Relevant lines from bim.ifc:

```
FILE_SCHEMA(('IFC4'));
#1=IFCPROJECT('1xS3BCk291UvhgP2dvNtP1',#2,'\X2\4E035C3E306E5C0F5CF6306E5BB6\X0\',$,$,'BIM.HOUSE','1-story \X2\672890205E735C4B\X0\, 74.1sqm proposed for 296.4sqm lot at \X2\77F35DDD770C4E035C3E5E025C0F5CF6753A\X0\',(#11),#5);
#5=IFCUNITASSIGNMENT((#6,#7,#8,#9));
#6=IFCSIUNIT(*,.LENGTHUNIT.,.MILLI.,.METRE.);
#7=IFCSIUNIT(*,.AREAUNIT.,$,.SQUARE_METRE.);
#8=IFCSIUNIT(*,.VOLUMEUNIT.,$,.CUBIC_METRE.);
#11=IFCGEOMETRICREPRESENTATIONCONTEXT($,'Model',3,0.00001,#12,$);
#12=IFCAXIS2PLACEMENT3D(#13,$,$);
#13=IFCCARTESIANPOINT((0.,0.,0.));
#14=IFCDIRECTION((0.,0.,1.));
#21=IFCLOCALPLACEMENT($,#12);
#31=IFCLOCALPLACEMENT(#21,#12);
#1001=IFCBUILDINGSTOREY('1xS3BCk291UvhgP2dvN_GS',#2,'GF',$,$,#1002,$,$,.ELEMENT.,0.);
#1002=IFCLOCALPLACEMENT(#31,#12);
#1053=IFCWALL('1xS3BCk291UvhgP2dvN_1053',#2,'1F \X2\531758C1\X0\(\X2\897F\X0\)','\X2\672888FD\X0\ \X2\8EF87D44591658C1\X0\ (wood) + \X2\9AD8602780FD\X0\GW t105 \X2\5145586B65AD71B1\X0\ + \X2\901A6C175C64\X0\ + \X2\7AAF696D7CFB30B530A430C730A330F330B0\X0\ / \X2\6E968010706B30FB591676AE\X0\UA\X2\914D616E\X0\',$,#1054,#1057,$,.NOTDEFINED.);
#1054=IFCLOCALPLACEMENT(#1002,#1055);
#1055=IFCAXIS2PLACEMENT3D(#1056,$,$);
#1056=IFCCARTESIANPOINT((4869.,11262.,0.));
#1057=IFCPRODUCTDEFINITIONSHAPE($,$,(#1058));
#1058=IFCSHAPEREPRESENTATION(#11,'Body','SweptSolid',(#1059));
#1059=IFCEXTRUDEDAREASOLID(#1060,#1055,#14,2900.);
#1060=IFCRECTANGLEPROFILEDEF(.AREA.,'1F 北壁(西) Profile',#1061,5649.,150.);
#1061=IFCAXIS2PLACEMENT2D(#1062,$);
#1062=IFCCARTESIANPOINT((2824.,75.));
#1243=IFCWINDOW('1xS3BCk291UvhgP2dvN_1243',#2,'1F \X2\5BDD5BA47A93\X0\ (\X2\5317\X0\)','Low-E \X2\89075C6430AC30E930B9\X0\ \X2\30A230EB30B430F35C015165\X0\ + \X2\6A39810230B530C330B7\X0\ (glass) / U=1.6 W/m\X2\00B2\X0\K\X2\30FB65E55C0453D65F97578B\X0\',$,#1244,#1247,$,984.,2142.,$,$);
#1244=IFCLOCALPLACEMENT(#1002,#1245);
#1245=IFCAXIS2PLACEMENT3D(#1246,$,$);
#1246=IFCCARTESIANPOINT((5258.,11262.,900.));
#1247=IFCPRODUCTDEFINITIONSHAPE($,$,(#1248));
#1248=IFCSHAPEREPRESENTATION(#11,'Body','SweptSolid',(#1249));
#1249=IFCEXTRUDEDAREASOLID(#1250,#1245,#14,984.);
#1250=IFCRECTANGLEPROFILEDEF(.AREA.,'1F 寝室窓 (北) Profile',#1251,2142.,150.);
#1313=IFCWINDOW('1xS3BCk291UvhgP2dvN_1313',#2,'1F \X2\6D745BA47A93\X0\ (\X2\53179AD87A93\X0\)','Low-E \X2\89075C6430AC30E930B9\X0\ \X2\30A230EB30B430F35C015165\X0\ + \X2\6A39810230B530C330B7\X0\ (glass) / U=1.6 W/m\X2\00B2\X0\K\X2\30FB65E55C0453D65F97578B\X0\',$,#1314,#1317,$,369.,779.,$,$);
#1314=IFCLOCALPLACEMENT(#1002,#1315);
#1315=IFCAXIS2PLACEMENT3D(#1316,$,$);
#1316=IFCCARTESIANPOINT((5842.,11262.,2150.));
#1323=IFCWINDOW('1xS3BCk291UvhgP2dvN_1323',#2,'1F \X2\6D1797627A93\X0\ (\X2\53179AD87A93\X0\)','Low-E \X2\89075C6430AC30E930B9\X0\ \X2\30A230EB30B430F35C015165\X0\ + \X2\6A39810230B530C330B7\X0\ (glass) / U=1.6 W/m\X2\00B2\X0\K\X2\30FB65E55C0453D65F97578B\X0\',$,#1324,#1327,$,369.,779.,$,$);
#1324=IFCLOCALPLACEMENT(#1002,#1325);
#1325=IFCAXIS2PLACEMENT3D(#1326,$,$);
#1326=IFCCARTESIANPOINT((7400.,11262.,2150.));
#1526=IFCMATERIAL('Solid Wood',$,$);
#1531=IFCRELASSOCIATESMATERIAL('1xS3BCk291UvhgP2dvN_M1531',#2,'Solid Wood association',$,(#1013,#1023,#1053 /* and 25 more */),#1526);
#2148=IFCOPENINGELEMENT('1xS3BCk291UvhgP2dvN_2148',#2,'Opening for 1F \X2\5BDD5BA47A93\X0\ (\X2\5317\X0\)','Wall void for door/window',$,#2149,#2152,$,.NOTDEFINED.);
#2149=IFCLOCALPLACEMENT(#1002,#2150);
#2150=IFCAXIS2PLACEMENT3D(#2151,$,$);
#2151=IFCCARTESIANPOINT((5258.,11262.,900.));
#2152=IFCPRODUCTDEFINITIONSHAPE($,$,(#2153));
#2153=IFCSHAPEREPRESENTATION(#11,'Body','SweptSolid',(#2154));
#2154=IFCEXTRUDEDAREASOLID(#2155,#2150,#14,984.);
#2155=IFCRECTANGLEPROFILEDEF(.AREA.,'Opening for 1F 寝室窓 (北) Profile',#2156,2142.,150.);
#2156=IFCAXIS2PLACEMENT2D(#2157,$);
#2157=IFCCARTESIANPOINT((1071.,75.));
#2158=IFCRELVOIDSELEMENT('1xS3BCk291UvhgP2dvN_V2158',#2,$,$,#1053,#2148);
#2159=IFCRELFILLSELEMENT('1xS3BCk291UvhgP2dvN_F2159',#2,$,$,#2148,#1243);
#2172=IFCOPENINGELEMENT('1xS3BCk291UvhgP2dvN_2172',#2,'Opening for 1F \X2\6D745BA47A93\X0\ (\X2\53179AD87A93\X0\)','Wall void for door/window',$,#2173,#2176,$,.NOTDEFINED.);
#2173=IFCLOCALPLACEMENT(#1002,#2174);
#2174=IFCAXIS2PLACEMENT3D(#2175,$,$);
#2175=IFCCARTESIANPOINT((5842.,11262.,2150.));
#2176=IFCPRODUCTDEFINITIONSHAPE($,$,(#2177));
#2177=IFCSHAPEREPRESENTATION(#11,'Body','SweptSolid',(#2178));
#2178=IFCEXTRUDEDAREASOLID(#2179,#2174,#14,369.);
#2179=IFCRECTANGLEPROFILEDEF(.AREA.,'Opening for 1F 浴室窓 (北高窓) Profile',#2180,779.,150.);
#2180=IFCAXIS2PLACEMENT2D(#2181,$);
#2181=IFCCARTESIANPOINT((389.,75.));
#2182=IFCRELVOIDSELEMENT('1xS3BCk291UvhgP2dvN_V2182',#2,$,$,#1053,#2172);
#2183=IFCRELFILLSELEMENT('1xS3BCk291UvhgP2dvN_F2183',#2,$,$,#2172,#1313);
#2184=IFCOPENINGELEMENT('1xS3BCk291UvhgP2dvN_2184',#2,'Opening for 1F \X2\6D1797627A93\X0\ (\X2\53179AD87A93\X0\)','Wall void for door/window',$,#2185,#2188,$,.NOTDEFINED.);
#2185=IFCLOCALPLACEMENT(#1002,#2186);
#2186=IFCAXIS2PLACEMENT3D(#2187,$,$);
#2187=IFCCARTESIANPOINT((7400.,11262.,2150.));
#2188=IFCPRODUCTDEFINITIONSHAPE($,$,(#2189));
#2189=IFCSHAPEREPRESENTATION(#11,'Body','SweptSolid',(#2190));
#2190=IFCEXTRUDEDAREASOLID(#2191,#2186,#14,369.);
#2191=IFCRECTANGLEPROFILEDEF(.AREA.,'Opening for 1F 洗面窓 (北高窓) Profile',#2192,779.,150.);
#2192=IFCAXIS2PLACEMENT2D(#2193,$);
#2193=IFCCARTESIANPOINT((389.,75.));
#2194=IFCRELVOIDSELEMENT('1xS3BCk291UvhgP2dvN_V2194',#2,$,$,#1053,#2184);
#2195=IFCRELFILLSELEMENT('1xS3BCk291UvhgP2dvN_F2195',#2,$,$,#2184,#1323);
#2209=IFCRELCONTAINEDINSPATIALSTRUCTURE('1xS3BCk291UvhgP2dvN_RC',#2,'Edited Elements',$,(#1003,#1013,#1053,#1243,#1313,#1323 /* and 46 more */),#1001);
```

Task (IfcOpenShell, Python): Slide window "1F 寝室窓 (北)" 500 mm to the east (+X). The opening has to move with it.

```python
import ifcopenshell
import ifcopenshell.api.geometry
import ifcopenshell.util.placement
import ifcopenshell.util.unit

model = ifcopenshell.open("bim.ifc")
unit_scale = ifcopenshell.util.unit.calculate_unit_scale(model)

window = model.by_guid("1xS3BCk291UvhgP2dvN_1243")
opening = window.FillsVoids[0].RelatingOpeningElement
wall = opening.VoidsElements[0].RelatingBuildingElement

wall_matrix = ifcopenshell.util.placement.get_local_placement(wall.ObjectPlacement)
shift = wall_matrix[:3, 0] * 0.5 / unit_scale
before = ifcopenshell.util.placement.get_local_placement(window.ObjectPlacement)[:3, 3].copy()

# The window is not placed relative to its opening, so move both.
for product in (opening, window):
    matrix = ifcopenshell.util.placement.get_local_placement(product.ObjectPlacement)
    matrix[:3, 3] += shift
    ifcopenshell.api.geometry.edit_object_placement(model, product=product, matrix=matrix, is_si=False)

after = ifcopenshell.util.placement.get_local_placement(window.ObjectPlacement)[:3, 3]
print("window moved by", (after - before).round(3) + 0.0)

model.write("bim_v2.ifc")
```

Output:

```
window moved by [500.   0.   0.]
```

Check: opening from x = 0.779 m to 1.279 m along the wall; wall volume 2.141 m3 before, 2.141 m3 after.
